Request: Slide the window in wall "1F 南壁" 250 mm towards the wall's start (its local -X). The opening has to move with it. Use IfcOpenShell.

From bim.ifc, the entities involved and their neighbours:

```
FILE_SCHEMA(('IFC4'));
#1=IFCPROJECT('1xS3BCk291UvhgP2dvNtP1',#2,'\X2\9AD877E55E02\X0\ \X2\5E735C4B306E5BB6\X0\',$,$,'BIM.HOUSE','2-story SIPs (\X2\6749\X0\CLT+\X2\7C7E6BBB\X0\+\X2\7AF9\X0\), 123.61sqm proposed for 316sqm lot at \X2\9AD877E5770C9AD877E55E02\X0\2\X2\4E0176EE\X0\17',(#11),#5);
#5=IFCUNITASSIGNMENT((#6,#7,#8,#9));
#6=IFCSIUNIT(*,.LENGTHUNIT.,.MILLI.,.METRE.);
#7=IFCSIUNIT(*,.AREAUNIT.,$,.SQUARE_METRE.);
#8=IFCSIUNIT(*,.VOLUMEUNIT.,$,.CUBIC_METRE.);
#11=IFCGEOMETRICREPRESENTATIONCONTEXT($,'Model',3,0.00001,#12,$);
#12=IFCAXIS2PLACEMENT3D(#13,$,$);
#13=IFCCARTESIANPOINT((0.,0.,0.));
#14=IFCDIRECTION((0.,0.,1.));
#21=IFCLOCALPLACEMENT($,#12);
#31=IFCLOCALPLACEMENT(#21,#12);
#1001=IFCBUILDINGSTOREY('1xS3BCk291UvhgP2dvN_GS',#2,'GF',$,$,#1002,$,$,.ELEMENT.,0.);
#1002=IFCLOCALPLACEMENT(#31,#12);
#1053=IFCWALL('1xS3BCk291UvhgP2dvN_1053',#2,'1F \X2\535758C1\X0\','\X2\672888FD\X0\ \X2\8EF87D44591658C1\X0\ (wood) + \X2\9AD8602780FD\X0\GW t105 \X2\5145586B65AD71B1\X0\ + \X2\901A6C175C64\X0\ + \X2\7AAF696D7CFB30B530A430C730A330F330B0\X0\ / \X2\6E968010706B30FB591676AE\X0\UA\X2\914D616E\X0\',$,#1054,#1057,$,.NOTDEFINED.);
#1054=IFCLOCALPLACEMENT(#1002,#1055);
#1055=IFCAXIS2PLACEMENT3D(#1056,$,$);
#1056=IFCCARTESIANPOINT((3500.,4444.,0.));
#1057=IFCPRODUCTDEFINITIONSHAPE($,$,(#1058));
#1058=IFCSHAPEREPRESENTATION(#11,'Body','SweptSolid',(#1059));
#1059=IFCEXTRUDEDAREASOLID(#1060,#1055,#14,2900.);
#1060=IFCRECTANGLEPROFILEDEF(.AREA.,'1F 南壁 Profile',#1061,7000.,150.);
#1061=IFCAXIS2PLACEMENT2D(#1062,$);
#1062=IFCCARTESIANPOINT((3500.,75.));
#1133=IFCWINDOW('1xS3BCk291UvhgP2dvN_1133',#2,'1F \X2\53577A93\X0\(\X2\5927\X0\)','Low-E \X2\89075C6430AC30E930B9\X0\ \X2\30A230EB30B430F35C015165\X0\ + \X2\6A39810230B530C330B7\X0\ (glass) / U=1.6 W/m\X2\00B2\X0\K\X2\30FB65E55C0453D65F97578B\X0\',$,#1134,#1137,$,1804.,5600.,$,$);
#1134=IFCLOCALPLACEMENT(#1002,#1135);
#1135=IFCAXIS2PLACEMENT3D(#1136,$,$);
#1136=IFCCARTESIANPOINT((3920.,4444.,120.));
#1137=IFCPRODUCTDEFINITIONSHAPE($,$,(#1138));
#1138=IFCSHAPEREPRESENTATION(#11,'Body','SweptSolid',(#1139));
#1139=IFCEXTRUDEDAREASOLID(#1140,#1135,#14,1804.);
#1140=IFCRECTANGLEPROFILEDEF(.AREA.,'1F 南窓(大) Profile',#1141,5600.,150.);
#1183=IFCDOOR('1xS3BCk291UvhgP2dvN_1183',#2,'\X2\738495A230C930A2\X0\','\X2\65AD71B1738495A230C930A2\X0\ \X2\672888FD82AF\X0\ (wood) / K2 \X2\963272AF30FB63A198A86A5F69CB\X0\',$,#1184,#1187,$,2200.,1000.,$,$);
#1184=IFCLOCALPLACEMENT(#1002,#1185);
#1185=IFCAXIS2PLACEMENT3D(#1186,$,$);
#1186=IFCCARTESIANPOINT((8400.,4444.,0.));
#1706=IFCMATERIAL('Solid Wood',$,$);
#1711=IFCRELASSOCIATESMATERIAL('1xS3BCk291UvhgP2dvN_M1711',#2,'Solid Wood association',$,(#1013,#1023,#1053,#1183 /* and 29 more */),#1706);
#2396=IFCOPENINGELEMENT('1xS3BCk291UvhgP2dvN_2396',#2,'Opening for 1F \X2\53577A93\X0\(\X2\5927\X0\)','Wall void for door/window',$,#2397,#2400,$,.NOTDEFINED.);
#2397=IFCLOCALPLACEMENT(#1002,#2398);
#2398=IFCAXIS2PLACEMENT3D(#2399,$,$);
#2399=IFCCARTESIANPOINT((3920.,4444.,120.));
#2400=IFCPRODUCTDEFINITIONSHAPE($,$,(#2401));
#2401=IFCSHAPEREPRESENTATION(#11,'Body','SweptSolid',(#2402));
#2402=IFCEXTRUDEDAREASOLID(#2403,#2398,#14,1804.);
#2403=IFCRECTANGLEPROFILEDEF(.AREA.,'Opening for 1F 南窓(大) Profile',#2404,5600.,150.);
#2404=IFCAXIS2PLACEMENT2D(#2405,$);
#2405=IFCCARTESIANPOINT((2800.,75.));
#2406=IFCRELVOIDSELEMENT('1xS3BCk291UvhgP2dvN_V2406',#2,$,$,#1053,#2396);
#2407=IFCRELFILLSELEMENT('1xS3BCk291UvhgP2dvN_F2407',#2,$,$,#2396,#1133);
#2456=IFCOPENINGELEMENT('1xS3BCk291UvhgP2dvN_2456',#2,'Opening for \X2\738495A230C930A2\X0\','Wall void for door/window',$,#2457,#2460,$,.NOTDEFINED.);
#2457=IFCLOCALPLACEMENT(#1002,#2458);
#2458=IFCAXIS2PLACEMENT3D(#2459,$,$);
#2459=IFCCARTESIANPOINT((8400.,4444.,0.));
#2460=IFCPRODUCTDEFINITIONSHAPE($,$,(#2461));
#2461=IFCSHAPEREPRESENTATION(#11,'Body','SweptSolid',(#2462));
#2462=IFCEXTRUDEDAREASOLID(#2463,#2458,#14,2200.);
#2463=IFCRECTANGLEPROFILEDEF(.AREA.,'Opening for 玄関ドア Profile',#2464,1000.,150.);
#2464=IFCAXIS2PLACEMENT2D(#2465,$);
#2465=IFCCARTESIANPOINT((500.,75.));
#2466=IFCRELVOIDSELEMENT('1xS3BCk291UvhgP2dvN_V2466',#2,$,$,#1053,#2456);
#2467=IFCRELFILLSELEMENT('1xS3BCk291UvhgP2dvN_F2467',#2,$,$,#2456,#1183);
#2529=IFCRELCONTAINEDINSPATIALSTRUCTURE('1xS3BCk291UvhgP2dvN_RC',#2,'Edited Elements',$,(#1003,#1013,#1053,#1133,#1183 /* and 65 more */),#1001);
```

```python
import ifcopenshell
import ifcopenshell.api.geometry
import ifcopenshell.util.placement
import ifcopenshell.util.unit

model = ifcopenshell.open("bim.ifc")
unit_scale = ifcopenshell.util.unit.calculate_unit_scale(model)

window = model.by_guid("1xS3BCk291UvhgP2dvN_1133")
opening = window.FillsVoids[0].RelatingOpeningElement
wall = opening.VoidsElements[0].RelatingBuildingElement

wall_matrix = ifcopenshell.util.placement.get_local_placement(wall.ObjectPlacement)
shift = wall_matrix[:3, 0] * -0.25 / unit_scale
before = ifcopenshell.util.placement.get_local_placement(window.ObjectPlacement)[:3, 3].copy()

# The window is not placed relative to its opening, so move both.
for product in (opening, window):
    matrix = ifcopenshell.util.placement.get_local_placement(product.ObjectPlacement)
    matrix[:3, 3] += shift
    ifcopenshell.api.geometry.edit_object_placement(model, product=product, matrix=matrix, is_si=False)

after = ifcopenshell.util.placement.get_local_placement(window.ObjectPlacement)[:3, 3]
print("window moved by", (after - before).round(3) + 0.0)

model.write("bim_edited.ifc")
```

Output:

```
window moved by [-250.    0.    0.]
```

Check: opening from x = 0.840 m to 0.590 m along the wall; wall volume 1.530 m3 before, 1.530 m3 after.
